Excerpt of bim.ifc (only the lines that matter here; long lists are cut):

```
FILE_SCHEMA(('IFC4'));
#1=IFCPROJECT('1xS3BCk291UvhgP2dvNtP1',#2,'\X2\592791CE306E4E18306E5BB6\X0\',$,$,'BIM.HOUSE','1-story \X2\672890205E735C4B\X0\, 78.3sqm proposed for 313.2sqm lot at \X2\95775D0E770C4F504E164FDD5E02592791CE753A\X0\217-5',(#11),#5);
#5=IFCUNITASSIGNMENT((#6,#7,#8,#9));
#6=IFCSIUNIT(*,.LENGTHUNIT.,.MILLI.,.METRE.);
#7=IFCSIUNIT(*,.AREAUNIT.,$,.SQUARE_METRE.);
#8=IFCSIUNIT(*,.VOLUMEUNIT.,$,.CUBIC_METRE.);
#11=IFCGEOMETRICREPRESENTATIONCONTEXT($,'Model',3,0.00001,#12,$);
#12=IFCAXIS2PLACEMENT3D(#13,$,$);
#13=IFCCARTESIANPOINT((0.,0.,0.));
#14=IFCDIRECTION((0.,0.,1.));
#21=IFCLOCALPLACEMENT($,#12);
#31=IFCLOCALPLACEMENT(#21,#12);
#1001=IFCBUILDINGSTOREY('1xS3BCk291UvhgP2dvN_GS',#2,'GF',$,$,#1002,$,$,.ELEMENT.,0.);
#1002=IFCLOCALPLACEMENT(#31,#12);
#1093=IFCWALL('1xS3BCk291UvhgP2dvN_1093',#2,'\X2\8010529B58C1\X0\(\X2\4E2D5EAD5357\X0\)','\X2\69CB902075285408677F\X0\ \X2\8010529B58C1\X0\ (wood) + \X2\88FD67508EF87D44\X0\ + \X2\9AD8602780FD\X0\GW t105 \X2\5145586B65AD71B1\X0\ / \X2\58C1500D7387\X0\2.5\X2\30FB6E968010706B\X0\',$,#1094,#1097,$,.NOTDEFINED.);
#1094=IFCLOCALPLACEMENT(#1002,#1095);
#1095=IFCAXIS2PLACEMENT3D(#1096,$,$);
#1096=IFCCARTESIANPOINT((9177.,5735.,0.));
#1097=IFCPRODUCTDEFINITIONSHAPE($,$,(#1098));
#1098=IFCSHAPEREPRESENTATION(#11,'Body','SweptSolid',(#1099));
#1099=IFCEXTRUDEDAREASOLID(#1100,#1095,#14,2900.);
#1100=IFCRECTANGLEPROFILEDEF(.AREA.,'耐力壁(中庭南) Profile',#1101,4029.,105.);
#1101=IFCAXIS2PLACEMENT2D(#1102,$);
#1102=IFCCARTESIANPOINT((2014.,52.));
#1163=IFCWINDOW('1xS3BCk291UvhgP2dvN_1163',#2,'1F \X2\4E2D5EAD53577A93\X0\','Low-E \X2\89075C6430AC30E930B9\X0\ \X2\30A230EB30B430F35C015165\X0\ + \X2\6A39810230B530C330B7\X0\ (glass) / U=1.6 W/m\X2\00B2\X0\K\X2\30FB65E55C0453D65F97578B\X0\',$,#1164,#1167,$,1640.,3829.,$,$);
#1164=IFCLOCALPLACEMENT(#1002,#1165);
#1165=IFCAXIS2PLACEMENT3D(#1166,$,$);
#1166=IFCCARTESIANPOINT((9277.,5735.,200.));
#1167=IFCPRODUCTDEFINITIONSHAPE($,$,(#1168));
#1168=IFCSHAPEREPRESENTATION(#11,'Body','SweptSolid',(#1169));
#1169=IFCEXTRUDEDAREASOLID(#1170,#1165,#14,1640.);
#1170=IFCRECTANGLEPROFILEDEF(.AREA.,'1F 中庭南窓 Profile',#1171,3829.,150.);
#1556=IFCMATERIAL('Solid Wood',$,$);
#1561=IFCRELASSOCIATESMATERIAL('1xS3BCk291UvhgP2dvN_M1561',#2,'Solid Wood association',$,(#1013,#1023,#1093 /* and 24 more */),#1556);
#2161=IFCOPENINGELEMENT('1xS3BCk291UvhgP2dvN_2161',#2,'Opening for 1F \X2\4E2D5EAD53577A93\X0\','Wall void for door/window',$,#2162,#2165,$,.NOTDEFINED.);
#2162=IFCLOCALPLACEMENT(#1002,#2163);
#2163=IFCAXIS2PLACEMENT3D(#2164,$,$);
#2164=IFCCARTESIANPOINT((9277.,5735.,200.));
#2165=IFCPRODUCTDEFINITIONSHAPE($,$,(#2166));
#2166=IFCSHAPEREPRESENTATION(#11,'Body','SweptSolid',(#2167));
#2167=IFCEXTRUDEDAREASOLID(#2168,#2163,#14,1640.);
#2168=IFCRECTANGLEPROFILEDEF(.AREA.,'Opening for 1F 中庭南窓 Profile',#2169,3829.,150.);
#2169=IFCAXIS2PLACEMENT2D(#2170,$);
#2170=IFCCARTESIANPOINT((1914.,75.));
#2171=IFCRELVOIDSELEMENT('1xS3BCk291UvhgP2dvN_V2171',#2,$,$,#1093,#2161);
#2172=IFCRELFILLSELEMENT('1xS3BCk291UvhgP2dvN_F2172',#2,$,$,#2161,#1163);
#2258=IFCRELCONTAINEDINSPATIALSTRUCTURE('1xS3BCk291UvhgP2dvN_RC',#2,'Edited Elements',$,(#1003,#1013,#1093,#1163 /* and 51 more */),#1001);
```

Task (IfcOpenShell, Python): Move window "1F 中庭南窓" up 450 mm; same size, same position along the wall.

```python
import numpy as np
import ifcopenshell
import ifcopenshell.api.geometry
import ifcopenshell.util.placement
import ifcopenshell.util.unit

model = ifcopenshell.open("bim.ifc")
unit_scale = ifcopenshell.util.unit.calculate_unit_scale(model)

window = model.by_guid("1xS3BCk291UvhgP2dvN_1163")
opening = window.FillsVoids[0].RelatingOpeningElement
dz = 450.0

shift = np.array([0.0, 0.0, dz])
# The window is not placed relative to its opening, so move both.
for product in (opening, window):
    matrix = ifcopenshell.util.placement.get_local_placement(product.ObjectPlacement)
    matrix[:3, 3] += shift
    ifcopenshell.api.geometry.edit_object_placement(model, product=product, matrix=matrix, is_si=False)

print(f"moved by {dz * unit_scale:+.3f} m")

model.write("bim_updated.ifc")
```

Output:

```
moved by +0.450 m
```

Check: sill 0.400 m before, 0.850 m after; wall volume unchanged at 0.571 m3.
